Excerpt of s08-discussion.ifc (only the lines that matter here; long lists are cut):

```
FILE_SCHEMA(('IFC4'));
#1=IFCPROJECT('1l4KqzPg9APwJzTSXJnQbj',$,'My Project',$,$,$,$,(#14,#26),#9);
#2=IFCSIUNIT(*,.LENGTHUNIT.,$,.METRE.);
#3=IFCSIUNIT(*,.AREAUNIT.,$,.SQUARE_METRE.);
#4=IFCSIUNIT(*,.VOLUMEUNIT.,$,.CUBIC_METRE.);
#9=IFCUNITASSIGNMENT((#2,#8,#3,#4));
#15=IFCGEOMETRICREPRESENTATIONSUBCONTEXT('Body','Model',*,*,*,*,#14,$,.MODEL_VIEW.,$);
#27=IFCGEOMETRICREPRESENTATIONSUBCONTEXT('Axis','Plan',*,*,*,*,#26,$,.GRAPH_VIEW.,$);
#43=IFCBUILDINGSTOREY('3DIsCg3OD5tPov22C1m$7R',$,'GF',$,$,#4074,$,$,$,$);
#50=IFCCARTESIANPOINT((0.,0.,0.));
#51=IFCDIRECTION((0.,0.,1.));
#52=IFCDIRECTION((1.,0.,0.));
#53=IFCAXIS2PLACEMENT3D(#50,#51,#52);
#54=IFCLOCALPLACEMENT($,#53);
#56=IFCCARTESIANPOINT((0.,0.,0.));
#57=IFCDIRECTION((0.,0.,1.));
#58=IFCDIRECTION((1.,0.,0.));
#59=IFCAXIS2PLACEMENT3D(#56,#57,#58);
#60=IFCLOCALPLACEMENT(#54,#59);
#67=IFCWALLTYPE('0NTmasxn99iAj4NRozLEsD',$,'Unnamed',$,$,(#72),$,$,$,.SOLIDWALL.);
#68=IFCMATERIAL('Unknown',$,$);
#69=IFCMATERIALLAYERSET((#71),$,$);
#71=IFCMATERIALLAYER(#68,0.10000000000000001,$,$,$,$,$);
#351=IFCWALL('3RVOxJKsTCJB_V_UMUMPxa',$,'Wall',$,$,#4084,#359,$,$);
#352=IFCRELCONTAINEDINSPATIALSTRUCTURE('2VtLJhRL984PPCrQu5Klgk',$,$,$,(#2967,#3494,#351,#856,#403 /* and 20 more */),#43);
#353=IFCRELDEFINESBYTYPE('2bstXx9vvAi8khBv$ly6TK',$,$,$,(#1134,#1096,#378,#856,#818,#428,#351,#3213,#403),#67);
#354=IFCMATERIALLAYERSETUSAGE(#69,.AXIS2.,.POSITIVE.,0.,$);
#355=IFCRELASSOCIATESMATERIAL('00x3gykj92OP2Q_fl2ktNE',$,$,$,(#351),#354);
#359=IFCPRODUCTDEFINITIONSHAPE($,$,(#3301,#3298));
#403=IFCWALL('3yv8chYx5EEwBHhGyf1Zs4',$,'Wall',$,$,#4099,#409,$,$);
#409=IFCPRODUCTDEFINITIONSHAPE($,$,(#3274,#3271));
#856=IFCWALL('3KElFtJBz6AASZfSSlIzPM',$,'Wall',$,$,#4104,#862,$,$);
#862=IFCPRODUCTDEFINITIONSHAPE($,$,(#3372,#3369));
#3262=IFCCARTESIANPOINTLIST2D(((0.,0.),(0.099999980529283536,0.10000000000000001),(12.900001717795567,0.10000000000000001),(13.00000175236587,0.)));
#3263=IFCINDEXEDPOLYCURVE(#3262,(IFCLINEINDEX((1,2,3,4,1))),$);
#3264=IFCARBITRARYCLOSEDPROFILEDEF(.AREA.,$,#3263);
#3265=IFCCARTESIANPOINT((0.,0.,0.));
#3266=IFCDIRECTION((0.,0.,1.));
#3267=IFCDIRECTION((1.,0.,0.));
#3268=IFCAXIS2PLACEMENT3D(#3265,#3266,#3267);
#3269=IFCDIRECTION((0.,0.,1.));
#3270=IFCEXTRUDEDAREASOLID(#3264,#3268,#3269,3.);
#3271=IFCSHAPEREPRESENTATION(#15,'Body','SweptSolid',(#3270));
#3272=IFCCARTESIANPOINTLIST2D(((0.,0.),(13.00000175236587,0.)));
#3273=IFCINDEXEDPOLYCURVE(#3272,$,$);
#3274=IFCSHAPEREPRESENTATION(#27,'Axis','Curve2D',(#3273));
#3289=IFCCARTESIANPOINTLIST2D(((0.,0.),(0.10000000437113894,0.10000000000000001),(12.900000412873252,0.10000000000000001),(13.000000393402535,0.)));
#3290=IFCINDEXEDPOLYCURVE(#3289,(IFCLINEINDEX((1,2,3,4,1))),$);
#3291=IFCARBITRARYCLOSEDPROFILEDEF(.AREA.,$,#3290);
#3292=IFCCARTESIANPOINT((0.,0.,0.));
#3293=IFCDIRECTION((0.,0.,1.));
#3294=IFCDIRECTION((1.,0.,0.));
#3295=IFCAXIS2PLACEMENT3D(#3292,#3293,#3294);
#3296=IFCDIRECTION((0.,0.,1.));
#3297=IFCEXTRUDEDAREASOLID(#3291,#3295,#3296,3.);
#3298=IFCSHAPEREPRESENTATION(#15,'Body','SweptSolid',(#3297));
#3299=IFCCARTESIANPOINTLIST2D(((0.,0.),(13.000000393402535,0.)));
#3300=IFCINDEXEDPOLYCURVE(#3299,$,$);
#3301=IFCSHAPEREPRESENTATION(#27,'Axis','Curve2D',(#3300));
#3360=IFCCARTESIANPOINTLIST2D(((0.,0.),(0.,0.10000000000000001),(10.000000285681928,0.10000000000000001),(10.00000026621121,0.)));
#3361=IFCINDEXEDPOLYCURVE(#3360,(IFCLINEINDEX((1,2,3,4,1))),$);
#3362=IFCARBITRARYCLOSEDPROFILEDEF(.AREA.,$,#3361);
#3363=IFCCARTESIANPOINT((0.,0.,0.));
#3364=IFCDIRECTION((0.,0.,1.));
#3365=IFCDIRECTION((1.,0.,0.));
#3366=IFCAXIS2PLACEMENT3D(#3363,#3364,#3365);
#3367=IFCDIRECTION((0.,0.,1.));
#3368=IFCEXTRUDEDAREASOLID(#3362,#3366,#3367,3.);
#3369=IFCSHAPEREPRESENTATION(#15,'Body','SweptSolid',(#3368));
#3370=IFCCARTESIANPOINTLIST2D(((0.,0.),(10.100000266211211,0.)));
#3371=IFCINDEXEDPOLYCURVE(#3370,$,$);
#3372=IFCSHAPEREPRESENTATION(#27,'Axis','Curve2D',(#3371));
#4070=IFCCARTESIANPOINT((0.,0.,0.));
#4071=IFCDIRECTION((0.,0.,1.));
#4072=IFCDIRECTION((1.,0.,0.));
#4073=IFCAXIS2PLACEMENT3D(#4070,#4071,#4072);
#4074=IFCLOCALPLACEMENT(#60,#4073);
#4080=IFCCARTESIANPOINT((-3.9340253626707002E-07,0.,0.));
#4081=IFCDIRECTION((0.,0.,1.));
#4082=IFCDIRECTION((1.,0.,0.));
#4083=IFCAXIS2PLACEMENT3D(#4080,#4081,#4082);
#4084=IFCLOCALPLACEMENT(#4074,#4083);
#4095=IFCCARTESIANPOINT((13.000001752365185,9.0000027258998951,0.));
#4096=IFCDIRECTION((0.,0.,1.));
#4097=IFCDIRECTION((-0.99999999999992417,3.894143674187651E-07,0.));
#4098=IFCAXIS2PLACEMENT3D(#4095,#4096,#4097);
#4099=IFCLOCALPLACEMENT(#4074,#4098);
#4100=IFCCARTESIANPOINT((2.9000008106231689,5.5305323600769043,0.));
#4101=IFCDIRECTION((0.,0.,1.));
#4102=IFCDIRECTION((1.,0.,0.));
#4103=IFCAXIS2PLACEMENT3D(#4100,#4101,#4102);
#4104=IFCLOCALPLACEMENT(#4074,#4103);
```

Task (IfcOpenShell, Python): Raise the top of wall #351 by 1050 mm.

```python
import ifcopenshell
import ifcopenshell.geom
import ifcopenshell.util.representation
import ifcopenshell.util.shape
import ifcopenshell.util.unit

model = ifcopenshell.open("s08-discussion.ifc")
unit_scale = ifcopenshell.util.unit.calculate_unit_scale(model)
settings = ifcopenshell.geom.settings()


def volume(element):
    """Net volume in cubic metres, openings subtracted."""
    shape = ifcopenshell.geom.create_shape(settings, element)
    return ifcopenshell.util.shape.get_volume(shape.geometry)


wall = model.by_guid("3RVOxJKsTCJB_V_UMUMPxa")
before = volume(wall)

body = ifcopenshell.util.representation.get_representation(wall, "Model", "Body")
solid = body.Items[0]
old_height = solid.Depth
solid.Depth += 1.05 / unit_scale
after = volume(wall)

print(f"height {old_height:g} -> {solid.Depth:g}, volume {before:.3f} -> {after:.3f} m3")

model.write("s08-discussion_updated.ifc")
```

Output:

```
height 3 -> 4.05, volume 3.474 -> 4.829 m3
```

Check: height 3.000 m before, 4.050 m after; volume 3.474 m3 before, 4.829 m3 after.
